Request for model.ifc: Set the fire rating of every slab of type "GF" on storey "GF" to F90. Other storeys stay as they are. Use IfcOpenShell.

First a look at what the model holds.

```python
import ifcopenshell
import ifcopenshell.util.element

model = ifcopenshell.open("model.ifc")
print(model.schema)
storey = next(s for s in model.by_type("IfcBuildingStorey") if s.Name == "GF")
slabs = [e for e in ifcopenshell.util.element.get_decomposition(storey) if e.is_a("IfcSlab")]
seen = {}
for e in slabs:
    element_type = ifcopenshell.util.element.get_type(e)
    key = (element_type.Name if element_type != e and element_type else None, ifcopenshell.util.element.get_pset(e, "Pset_SlabCommon", "FireRating"))
    seen[key] = seen.get(key, 0) + 1
for (name, value), count in sorted(seen.items(), key=str):
    print(count, "x", name, "|", value)
```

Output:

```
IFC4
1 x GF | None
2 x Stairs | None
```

```python
import ifcopenshell
import ifcopenshell.api.pset
import ifcopenshell.util.element

model = ifcopenshell.open("model.ifc")

storey = next(s for s in model.by_type("IfcBuildingStorey") if s.Name == "GF")
slabs = [e for e in ifcopenshell.util.element.get_decomposition(storey) if e.is_a("IfcSlab")]

count = 0
for e in slabs:
    element_type = ifcopenshell.util.element.get_type(e)
    if element_type in (None, e) or element_type.Name != "GF":
        continue
    # add_pset returns the element's existing set when there is one.
    pset = ifcopenshell.api.pset.add_pset(model, product=e, name="Pset_SlabCommon")
    ifcopenshell.api.pset.edit_pset(model, pset=pset, properties={"FireRating": "F90"})
    count += 1

print(count, "slabs updated")

model.write("model_v2.ifc")
```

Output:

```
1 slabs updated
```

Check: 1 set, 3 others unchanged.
